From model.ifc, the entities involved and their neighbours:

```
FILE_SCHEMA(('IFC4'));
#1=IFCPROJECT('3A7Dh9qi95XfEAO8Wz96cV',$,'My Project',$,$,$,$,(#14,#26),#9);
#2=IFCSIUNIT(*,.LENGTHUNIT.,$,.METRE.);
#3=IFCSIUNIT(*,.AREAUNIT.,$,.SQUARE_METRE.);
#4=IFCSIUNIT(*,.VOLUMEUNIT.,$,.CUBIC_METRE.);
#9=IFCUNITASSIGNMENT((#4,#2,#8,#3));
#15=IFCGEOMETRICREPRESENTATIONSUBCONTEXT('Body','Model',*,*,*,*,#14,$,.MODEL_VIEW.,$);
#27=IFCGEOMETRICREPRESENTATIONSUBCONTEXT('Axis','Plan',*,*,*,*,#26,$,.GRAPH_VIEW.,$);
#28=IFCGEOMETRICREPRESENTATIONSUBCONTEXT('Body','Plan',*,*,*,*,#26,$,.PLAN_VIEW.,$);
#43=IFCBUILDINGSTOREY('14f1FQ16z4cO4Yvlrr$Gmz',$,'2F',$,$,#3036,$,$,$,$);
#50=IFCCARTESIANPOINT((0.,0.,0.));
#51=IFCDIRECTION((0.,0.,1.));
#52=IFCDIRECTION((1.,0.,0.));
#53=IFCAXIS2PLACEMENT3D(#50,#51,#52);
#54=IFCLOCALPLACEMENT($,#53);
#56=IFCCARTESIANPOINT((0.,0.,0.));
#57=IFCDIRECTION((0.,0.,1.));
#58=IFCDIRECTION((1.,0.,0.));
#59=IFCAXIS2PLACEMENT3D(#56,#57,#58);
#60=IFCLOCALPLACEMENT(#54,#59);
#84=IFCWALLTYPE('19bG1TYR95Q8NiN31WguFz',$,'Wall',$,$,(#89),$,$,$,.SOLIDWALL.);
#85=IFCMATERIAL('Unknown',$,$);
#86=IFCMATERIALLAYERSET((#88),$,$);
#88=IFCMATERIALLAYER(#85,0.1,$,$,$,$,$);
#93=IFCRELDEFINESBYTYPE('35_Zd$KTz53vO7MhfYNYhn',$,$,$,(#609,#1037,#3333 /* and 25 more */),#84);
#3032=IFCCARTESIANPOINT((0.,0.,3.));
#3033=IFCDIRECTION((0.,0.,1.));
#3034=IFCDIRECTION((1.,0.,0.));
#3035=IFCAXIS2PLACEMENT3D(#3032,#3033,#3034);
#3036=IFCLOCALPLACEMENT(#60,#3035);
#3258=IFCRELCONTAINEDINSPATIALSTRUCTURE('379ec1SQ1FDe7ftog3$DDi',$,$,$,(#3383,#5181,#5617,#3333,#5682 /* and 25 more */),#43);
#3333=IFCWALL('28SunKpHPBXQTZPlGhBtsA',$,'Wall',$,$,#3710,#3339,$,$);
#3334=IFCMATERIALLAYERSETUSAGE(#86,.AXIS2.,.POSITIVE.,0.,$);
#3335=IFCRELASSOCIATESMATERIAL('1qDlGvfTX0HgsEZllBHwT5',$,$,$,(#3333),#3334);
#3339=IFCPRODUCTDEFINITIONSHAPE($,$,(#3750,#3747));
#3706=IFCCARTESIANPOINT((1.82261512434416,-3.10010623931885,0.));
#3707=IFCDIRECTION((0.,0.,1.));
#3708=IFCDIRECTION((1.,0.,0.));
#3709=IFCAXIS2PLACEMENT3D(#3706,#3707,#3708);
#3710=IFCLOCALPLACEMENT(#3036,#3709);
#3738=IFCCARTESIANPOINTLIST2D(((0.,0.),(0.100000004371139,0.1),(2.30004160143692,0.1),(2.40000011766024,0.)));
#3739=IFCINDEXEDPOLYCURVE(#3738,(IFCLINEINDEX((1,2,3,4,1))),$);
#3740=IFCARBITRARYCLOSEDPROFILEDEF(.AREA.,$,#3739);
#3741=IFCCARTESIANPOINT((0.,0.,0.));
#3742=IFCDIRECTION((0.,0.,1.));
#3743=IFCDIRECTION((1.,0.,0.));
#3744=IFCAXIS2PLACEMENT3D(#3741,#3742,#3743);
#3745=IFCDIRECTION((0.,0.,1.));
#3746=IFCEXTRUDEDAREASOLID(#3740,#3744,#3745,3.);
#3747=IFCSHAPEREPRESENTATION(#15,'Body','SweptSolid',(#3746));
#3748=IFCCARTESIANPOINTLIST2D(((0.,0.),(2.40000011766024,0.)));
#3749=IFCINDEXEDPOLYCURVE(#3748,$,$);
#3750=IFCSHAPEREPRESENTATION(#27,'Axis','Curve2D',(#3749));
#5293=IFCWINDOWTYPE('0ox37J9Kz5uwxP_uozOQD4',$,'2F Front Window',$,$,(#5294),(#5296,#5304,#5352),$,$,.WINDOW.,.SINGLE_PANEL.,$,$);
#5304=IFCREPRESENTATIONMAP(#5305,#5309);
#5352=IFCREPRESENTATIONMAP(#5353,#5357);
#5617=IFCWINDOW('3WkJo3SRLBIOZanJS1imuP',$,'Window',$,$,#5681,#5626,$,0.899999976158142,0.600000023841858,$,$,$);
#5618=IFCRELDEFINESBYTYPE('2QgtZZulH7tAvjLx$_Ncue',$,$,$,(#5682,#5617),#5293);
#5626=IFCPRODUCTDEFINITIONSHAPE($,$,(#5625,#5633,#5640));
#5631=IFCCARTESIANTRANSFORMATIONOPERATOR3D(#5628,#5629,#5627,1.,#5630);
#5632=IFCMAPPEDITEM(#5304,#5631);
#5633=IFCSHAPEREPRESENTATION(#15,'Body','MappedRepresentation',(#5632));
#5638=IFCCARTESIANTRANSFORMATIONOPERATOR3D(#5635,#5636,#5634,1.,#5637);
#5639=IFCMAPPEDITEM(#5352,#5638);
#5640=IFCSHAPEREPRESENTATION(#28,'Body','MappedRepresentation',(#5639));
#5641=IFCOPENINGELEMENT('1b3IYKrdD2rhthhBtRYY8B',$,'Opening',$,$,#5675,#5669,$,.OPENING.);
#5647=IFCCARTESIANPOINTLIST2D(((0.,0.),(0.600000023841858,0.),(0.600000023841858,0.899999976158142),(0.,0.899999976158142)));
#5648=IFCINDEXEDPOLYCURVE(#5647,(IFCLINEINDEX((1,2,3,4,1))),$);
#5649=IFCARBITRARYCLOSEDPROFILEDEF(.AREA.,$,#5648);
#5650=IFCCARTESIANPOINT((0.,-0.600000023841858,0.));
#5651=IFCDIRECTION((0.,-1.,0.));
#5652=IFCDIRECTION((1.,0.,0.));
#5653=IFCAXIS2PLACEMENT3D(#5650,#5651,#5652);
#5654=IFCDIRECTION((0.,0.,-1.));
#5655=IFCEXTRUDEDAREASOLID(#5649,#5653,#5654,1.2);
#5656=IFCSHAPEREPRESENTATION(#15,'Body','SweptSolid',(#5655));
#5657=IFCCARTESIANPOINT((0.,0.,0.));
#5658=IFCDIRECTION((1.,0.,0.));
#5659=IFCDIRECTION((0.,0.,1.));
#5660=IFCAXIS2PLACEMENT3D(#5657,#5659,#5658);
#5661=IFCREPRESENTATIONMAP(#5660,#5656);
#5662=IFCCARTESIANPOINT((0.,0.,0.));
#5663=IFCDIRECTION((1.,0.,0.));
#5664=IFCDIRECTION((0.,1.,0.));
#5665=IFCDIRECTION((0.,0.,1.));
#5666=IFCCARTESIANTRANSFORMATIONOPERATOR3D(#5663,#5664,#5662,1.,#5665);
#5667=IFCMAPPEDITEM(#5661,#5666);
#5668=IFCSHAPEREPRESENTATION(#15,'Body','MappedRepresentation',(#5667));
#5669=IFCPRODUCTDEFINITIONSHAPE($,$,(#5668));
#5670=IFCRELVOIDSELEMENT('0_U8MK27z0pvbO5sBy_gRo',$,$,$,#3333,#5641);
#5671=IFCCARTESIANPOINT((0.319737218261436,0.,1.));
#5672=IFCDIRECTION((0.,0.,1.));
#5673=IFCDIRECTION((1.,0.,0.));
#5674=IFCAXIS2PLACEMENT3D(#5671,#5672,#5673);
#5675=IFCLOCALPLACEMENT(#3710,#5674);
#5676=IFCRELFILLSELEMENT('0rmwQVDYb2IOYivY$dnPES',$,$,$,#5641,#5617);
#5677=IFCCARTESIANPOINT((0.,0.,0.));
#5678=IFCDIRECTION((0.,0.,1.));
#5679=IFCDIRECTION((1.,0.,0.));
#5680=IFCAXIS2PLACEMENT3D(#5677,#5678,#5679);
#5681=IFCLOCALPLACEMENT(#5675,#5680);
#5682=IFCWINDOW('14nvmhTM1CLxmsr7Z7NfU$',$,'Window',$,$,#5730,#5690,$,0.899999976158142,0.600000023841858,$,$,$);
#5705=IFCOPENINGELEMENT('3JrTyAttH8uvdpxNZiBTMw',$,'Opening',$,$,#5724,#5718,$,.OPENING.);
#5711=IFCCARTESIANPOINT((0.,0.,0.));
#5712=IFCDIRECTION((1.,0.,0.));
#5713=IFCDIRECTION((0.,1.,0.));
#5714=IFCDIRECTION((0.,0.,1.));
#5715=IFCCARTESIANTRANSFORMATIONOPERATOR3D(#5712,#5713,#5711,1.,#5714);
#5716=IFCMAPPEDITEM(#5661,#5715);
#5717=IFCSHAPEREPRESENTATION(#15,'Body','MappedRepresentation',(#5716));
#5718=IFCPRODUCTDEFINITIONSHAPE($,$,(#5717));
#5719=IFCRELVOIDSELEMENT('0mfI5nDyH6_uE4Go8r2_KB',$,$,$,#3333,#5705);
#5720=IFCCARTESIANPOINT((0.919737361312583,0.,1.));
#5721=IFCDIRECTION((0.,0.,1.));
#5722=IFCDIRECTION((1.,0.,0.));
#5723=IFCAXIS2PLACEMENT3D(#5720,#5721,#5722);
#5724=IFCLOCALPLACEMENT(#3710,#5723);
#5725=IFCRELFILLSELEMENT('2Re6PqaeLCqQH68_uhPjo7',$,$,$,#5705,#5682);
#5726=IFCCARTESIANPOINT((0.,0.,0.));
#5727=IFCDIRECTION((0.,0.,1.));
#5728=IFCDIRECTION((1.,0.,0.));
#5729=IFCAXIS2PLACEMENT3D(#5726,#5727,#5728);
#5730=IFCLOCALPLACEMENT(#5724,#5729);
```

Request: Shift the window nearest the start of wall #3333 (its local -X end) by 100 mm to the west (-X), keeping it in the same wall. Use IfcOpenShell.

```python
import ifcopenshell
import ifcopenshell.api.geometry
import ifcopenshell.util.placement
import ifcopenshell.util.unit

model = ifcopenshell.open("model.ifc")
unit_scale = ifcopenshell.util.unit.calculate_unit_scale(model)

window = model.by_guid("3WkJo3SRLBIOZanJS1imuP")
opening = window.FillsVoids[0].RelatingOpeningElement
wall = opening.VoidsElements[0].RelatingBuildingElement

wall_matrix = ifcopenshell.util.placement.get_local_placement(wall.ObjectPlacement)
shift = wall_matrix[:3, 0] * -0.1 / unit_scale
before = ifcopenshell.util.placement.get_local_placement(window.ObjectPlacement)[:3, 3].copy()

# The window is placed relative to its opening, so it follows when the opening moves.
matrix = ifcopenshell.util.placement.get_local_placement(opening.ObjectPlacement)
matrix[:3, 3] += shift
ifcopenshell.api.geometry.edit_object_placement(
    model, product=opening, matrix=matrix, is_si=False, should_transform_children=True
)

after = ifcopenshell.util.placement.get_local_placement(window.ObjectPlacement)[:3, 3]
print("window moved by", (after - before).round(3) + 0.0)

model.write("model-out.ifc")
```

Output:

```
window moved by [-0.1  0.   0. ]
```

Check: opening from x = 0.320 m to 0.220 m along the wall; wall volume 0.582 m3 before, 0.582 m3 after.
